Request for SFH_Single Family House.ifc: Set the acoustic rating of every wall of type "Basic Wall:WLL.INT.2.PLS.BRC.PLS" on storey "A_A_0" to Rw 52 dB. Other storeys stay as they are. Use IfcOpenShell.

First a look at what the model holds.

```python
import ifcopenshell
import ifcopenshell.util.element

model = ifcopenshell.open("SFH_Single Family House.ifc")
print(model.schema)
storey = next(s for s in model.by_type("IfcBuildingStorey") if s.Name == "A_A_0")
walls = [e for e in ifcopenshell.util.element.get_decomposition(storey) if e.is_a("IfcWall")]
seen = {}
for e in walls:
    element_type = ifcopenshell.util.element.get_type(e)
    key = (element_type.Name if element_type != e and element_type else None, ifcopenshell.util.element.get_pset(e, "Pset_WallCommon", "AcousticRating"))
    seen[key] = seen.get(key, 0) + 1
for (name, value), count in sorted(seen.items(), key=str):
    print(count, "x", name, "|", value)
```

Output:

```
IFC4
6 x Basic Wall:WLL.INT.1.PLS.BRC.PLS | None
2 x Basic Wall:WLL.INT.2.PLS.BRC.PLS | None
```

```python
import ifcopenshell
import ifcopenshell.api.pset
import ifcopenshell.util.element

model = ifcopenshell.open("SFH_Single Family House.ifc")

storey = next(s for s in model.by_type("IfcBuildingStorey") if s.Name == "A_A_0")
walls = [e for e in ifcopenshell.util.element.get_decomposition(storey) if e.is_a("IfcWall")]

count = 0
for e in walls:
    element_type = ifcopenshell.util.element.get_type(e)
    if element_type in (None, e) or element_type.Name != "Basic Wall:WLL.INT.2.PLS.BRC.PLS":
        continue
    # add_pset returns the element's existing set when there is one.
    pset = ifcopenshell.api.pset.add_pset(model, product=e, name="Pset_WallCommon")
    ifcopenshell.api.pset.edit_pset(model, pset=pset, properties={"AcousticRating": "Rw 52 dB"})
    count += 1

print(count, "walls updated")

model.write("SFH_Single Family House_edited.ifc")
```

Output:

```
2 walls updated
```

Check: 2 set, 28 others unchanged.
